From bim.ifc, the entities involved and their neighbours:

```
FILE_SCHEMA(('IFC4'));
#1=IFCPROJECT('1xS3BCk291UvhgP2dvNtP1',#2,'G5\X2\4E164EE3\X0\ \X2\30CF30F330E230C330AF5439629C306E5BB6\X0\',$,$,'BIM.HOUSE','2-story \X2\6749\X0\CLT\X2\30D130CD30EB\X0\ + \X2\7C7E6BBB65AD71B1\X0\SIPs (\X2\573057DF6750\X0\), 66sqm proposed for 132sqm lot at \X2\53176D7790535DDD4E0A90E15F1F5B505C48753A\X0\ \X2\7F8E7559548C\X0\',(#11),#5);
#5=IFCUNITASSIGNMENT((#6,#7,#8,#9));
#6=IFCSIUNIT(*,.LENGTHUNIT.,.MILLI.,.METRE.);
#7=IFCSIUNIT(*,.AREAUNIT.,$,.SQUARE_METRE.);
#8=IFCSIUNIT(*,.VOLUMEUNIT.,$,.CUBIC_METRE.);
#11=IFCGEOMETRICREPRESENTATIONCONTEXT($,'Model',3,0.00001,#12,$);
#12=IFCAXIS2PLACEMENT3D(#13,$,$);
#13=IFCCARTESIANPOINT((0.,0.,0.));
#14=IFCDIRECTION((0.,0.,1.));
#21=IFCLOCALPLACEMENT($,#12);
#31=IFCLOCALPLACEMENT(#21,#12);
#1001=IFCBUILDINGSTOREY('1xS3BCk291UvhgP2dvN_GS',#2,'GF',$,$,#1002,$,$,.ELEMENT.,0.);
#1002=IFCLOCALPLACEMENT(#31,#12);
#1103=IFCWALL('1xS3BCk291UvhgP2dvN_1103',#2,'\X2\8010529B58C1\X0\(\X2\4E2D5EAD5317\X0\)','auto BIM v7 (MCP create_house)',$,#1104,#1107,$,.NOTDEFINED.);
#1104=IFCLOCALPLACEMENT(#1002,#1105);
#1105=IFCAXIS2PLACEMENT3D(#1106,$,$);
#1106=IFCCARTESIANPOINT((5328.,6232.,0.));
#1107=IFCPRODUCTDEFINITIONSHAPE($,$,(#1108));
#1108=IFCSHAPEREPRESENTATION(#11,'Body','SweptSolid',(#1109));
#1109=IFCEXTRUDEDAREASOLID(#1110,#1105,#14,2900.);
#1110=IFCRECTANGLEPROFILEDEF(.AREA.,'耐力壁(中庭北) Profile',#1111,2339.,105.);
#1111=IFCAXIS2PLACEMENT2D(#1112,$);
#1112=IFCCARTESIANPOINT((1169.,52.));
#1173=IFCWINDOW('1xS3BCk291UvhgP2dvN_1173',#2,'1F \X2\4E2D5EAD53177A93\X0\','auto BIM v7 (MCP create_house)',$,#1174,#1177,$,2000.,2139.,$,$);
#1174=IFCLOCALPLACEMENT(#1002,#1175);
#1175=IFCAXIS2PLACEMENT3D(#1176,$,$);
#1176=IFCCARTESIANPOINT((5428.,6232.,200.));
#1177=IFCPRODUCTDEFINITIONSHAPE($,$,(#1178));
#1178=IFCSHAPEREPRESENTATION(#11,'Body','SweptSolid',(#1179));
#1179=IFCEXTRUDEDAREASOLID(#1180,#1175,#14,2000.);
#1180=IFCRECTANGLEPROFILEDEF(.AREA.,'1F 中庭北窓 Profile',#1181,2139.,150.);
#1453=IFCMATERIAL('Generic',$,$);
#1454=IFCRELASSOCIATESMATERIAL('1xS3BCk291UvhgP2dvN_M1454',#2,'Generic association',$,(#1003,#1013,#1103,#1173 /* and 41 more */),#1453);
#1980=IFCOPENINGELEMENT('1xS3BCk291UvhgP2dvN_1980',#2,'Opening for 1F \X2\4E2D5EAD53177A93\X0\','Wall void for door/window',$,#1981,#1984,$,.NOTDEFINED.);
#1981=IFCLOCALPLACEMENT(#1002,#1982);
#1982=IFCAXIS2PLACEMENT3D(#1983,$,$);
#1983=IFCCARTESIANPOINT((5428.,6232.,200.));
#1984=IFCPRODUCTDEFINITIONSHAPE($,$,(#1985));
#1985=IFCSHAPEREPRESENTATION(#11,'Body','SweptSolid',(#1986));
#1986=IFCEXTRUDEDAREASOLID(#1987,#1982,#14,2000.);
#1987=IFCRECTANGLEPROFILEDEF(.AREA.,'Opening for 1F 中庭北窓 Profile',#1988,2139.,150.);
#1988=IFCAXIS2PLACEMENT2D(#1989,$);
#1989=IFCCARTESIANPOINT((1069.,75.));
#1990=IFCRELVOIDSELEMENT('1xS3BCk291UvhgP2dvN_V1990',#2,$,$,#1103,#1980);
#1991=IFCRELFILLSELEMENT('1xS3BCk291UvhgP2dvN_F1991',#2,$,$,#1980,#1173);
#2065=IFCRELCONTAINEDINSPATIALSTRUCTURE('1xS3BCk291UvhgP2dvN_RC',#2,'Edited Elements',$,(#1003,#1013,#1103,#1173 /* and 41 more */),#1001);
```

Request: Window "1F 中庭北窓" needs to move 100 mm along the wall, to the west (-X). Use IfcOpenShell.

```python
import ifcopenshell
import ifcopenshell.api.geometry
import ifcopenshell.util.placement

model = ifcopenshell.open("bim.ifc")

window = model.by_guid("1xS3BCk291UvhgP2dvN_1173")
opening = window.FillsVoids[0].RelatingOpeningElement
wall = opening.VoidsElements[0].RelatingBuildingElement

wall_matrix = ifcopenshell.util.placement.get_local_placement(wall.ObjectPlacement)
shift = wall_matrix[:3, 0] * -100.0
before = ifcopenshell.util.placement.get_local_placement(window.ObjectPlacement)[:3, 3].copy()

# The window is not placed relative to its opening, so move both.
for product in (opening, window):
    matrix = ifcopenshell.util.placement.get_local_placement(product.ObjectPlacement)
    matrix[:3, 3] += shift
    ifcopenshell.api.geometry.edit_object_placement(model, product=product, matrix=matrix, is_si=False)

after = ifcopenshell.util.placement.get_local_placement(window.ObjectPlacement)[:3, 3]
print("window moved by", (after - before).round(3) + 0.0)

model.write("bim_updated.ifc")
```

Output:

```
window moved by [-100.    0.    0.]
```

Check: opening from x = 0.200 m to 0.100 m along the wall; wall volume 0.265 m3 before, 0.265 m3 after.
